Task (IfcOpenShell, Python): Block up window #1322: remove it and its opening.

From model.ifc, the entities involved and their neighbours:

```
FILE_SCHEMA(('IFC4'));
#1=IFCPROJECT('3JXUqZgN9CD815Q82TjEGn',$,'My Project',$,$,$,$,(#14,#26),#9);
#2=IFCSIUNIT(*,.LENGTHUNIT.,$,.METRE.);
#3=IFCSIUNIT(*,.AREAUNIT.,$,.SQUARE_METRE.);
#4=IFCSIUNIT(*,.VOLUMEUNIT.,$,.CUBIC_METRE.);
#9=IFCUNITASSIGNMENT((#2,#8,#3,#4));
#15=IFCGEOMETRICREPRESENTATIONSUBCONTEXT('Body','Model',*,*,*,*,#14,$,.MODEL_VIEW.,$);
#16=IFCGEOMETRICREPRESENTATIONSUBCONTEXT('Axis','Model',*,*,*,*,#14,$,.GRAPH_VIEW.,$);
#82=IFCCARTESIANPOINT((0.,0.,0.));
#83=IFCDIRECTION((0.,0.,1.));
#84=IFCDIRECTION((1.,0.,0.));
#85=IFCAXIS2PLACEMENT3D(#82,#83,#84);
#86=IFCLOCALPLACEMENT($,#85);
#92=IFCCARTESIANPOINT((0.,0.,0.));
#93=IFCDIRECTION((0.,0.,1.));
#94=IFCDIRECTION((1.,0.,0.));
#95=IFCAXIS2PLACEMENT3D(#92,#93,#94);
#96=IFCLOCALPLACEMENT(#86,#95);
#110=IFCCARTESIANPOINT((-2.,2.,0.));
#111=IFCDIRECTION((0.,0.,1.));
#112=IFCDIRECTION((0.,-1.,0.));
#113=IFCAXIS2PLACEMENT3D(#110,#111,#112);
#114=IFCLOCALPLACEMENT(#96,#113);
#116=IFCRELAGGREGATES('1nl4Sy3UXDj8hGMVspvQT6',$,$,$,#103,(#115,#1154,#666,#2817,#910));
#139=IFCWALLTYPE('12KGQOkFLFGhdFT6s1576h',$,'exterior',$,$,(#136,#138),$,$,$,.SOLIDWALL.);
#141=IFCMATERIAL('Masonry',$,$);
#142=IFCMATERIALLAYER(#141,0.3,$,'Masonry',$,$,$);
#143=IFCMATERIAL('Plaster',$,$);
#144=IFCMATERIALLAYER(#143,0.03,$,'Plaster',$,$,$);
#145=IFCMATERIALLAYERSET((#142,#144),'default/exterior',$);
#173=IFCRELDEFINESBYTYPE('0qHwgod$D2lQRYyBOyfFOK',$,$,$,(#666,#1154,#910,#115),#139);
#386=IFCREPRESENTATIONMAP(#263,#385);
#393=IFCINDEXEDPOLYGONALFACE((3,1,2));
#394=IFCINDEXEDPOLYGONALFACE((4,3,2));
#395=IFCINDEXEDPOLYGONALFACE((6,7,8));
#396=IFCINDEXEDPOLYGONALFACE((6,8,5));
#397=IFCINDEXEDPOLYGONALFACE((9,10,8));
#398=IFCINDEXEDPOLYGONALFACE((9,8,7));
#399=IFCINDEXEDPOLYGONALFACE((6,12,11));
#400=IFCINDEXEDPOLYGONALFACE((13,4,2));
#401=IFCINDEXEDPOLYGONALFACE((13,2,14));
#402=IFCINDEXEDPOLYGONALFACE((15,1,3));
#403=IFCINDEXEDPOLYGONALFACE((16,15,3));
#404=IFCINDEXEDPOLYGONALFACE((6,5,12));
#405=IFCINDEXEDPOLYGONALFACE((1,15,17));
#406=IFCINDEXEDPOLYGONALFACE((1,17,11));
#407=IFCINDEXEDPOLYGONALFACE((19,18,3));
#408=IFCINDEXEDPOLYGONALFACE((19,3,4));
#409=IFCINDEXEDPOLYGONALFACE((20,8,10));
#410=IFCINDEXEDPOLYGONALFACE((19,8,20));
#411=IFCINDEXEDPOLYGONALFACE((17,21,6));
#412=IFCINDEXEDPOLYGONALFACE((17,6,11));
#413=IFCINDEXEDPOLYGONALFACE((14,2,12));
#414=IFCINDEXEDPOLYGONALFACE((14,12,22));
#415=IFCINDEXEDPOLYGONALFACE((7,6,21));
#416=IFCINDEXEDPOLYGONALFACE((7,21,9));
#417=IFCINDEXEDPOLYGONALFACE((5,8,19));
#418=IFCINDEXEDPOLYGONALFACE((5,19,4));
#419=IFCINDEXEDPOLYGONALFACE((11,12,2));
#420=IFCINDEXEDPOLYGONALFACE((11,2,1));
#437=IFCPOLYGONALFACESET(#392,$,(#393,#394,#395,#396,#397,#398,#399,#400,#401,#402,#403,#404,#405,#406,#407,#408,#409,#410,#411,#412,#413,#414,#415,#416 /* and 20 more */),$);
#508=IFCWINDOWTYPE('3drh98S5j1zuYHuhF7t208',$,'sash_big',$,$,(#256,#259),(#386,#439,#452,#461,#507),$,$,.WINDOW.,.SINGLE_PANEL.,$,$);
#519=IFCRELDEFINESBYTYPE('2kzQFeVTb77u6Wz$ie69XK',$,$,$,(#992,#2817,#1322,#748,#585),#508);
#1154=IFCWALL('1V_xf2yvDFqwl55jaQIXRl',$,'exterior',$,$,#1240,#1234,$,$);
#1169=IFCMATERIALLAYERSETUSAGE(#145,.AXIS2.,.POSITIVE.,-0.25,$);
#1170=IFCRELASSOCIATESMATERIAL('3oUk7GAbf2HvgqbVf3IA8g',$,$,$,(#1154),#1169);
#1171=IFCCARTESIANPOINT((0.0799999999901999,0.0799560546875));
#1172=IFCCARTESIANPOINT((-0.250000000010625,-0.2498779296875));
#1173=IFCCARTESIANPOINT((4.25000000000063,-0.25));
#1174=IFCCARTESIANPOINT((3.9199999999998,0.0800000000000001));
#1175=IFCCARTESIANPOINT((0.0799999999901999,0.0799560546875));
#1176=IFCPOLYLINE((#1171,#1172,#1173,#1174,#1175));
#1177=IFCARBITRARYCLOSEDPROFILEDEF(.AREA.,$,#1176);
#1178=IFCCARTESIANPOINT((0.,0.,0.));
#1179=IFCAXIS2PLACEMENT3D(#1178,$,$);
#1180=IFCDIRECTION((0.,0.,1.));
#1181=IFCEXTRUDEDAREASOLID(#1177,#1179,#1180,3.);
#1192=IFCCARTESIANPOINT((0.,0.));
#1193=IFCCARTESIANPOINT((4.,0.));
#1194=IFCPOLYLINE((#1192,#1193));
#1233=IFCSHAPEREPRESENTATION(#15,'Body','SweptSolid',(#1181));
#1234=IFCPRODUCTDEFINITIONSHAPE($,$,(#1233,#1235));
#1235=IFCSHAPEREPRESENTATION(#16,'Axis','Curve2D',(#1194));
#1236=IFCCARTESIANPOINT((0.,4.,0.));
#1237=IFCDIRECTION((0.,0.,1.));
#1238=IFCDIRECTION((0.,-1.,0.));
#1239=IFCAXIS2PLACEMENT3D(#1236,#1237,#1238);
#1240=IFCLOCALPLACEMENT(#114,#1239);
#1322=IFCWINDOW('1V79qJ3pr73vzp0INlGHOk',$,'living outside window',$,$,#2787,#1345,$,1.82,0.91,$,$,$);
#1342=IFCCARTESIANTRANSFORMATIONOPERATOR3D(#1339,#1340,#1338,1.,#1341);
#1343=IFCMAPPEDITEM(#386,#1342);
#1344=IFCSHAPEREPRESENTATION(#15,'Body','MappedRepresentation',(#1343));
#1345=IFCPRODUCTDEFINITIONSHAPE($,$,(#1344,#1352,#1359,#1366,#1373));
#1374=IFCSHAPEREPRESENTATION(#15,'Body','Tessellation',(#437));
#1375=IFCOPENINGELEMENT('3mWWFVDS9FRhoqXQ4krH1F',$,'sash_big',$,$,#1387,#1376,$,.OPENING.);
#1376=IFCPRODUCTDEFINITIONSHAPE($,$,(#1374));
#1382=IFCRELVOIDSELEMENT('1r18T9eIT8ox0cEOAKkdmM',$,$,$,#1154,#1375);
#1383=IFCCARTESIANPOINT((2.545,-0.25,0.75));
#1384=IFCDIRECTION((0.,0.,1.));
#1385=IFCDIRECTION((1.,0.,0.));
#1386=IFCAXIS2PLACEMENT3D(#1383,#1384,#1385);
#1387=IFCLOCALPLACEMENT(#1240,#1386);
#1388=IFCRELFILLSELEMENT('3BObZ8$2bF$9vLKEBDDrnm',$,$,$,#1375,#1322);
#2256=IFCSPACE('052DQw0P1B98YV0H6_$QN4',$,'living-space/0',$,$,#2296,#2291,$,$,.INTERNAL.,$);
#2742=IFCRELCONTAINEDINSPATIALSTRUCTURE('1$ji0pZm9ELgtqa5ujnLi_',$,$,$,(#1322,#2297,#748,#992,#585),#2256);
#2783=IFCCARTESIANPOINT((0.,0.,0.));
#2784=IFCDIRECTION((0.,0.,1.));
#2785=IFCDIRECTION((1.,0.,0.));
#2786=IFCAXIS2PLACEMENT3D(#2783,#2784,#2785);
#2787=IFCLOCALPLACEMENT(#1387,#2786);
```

```python
import ifcopenshell
import ifcopenshell.api.feature
import ifcopenshell.api.root
import ifcopenshell.geom
import ifcopenshell.util.shape

model = ifcopenshell.open("model.ifc")
settings = ifcopenshell.geom.settings()


def volume(element):
    """Net volume in cubic metres, openings subtracted."""
    shape = ifcopenshell.geom.create_shape(settings, element)
    return ifcopenshell.util.shape.get_volume(shape.geometry)


window = model.by_guid("1V79qJ3pr73vzp0INlGHOk")
opening = window.FillsVoids[0].RelatingOpeningElement
wall = opening.VoidsElements[0].RelatingBuildingElement
before = volume(wall)

ifcopenshell.api.root.remove_product(model, product=window)
ifcopenshell.api.feature.remove_feature(model, feature=opening)

after = volume(wall)

print(f"wall volume {before:.3f} -> {after:.3f} m3")

model.write("model_v2.ifc")
```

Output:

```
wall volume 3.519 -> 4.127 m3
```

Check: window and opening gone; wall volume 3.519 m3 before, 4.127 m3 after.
